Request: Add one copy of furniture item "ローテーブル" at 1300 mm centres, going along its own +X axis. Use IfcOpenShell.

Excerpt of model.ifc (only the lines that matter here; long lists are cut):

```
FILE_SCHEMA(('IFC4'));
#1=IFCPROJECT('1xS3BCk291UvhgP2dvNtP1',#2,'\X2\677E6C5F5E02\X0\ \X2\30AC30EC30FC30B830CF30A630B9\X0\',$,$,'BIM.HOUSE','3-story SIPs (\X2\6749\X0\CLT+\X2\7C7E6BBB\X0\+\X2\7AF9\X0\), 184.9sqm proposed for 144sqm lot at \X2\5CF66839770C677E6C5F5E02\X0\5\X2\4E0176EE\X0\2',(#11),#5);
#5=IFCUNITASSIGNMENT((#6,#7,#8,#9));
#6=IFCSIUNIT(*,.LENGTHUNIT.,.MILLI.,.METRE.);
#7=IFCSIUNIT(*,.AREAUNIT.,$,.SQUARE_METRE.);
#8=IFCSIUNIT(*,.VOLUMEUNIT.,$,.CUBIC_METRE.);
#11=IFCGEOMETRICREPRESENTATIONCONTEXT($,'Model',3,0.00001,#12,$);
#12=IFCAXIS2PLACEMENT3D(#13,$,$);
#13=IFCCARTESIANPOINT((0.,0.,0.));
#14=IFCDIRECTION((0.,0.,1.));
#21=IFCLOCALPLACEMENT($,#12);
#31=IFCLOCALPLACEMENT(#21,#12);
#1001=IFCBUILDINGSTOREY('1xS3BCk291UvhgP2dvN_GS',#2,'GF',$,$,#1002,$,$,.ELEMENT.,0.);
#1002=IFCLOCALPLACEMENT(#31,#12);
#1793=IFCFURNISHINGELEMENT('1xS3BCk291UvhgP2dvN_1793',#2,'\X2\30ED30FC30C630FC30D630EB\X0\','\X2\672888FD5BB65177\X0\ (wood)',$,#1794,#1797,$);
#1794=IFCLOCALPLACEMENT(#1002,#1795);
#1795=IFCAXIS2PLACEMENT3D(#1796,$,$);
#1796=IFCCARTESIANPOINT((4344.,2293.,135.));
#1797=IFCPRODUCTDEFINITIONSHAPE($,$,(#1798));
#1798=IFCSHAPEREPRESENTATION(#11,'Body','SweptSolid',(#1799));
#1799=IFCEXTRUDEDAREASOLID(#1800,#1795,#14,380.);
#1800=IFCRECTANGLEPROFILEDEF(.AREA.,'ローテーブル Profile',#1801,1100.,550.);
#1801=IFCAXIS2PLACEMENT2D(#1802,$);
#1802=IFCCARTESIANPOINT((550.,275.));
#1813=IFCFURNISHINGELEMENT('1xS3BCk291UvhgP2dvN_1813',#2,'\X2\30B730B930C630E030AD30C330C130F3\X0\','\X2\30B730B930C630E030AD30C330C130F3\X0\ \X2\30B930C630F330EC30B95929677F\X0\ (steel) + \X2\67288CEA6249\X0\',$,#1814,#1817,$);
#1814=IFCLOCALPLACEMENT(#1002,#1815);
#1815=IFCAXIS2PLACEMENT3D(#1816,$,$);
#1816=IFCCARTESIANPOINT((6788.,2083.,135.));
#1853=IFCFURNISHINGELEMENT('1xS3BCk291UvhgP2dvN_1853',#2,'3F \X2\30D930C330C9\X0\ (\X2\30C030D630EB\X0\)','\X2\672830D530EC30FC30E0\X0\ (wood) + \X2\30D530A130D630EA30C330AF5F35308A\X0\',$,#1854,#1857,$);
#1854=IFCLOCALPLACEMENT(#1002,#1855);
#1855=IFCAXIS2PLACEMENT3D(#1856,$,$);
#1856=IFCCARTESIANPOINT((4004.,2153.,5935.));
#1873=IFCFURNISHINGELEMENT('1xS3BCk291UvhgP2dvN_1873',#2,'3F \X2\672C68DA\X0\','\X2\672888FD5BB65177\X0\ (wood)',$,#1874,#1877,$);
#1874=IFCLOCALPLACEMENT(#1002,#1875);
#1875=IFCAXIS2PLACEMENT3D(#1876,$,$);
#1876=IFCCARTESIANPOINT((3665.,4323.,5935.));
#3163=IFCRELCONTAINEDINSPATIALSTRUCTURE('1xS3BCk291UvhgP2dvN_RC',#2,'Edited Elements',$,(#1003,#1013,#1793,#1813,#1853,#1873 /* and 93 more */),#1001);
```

```python
import ifcopenshell
import ifcopenshell.api.geometry
import ifcopenshell.api.root
import ifcopenshell.util.element
import ifcopenshell.util.placement

model = ifcopenshell.open("model.ifc")


def reuse_history(source, copy):
    """copy_class also copies each property set's owner history, people and application; keep the originals."""
    for rel in copy.IsDefinedBy:
        if rel.is_a("IfcRelDefinesByProperties") and (history := rel.RelatingPropertyDefinition.OwnerHistory):
            rel.RelatingPropertyDefinition.OwnerHistory = source.OwnerHistory
            ifcopenshell.util.element.remove_deep2(model, history)


source = model.by_guid("1xS3BCk291UvhgP2dvN_1793")
base = ifcopenshell.util.placement.get_local_placement(source.ObjectPlacement)
step = base[:3, 0] * 1300.0

for i in range(1, 2):
    copy = ifcopenshell.api.root.copy_class(model, product=source)
    copy.Representation = ifcopenshell.util.element.copy_deep(
        model, source.Representation, exclude=["IfcGeometricRepresentationContext", "IfcRepresentationMap"]
    )
    reuse_history(source, copy)
    matrix = base.copy()
    matrix[:3, 3] += i * step
    print("added at", matrix[:3, 3].round(3) + 0.0)
    ifcopenshell.api.geometry.edit_object_placement(model, product=copy, matrix=matrix, is_si=False)

model.write("model_updated.ifc")
```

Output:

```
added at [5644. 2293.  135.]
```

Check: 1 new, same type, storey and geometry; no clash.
